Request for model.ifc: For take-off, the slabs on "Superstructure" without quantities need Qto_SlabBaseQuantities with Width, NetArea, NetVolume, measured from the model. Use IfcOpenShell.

First a look at what the model holds.

```python
import ifcopenshell
import ifcopenshell.util.element
import ifcopenshell.util.unit

model = ifcopenshell.open("model.ifc")
print(model.schema)
for unit_type in ("LENGTHUNIT", "AREAUNIT", "VOLUMEUNIT"):
    print(unit_type, ifcopenshell.util.unit.calculate_unit_scale(model, unit_type))
storey = next(s for s in model.by_type("IfcBuildingStorey") if s.Name == "Superstructure")
slabs = [e for e in ifcopenshell.util.element.get_decomposition(storey) if e.is_a("IfcSlab")]
for e in sorted(slabs, key=lambda e: e.id()):
    print(e.id(), e.is_a(), e.Name, list(ifcopenshell.util.element.get_psets(e, qtos_only=True)), sep=" | ")
```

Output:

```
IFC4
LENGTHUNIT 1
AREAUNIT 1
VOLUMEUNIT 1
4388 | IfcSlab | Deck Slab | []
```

```python
import ifcopenshell
import ifcopenshell.api.pset
import ifcopenshell.geom
import ifcopenshell.util.element
import ifcopenshell.util.shape
import ifcopenshell.util.unit

model = ifcopenshell.open("model.ifc")
unit_scale = ifcopenshell.util.unit.calculate_unit_scale(model)
area_scale = ifcopenshell.util.unit.calculate_unit_scale(model, "AREAUNIT")
volume_scale = ifcopenshell.util.unit.calculate_unit_scale(model, "VOLUMEUNIT")
settings = ifcopenshell.geom.settings()

storey = next(s for s in model.by_type("IfcBuildingStorey") if s.Name == "Superstructure")
slabs = [e for e in ifcopenshell.util.element.get_decomposition(storey) if e.is_a("IfcSlab")]

for e in sorted(slabs, key=lambda e: e.id()):
    if ifcopenshell.util.element.get_psets(e, qtos_only=True, should_inherit=False):
        continue
    # Geometry comes back in metres, in the element's own axes.
    shape = ifcopenshell.geom.create_shape(settings, e)
    values = {
        "Width": ifcopenshell.util.shape.get_z(shape.geometry) / unit_scale,
        "NetArea": ifcopenshell.util.shape.get_footprint_area(shape.geometry) / area_scale,
        "NetVolume": ifcopenshell.util.shape.get_volume(shape.geometry) / volume_scale,
    }
    qto = ifcopenshell.api.pset.add_qto(model, product=e, name="Qto_SlabBaseQuantities")
    ifcopenshell.api.pset.edit_qto(model, qto=qto, properties=values)
    print(e.id(), {k: round(v, 3) for k, v in values.items()})

model.write("model_rev.ifc")
```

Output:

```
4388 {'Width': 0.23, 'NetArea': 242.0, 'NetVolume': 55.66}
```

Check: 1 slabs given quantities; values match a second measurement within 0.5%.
